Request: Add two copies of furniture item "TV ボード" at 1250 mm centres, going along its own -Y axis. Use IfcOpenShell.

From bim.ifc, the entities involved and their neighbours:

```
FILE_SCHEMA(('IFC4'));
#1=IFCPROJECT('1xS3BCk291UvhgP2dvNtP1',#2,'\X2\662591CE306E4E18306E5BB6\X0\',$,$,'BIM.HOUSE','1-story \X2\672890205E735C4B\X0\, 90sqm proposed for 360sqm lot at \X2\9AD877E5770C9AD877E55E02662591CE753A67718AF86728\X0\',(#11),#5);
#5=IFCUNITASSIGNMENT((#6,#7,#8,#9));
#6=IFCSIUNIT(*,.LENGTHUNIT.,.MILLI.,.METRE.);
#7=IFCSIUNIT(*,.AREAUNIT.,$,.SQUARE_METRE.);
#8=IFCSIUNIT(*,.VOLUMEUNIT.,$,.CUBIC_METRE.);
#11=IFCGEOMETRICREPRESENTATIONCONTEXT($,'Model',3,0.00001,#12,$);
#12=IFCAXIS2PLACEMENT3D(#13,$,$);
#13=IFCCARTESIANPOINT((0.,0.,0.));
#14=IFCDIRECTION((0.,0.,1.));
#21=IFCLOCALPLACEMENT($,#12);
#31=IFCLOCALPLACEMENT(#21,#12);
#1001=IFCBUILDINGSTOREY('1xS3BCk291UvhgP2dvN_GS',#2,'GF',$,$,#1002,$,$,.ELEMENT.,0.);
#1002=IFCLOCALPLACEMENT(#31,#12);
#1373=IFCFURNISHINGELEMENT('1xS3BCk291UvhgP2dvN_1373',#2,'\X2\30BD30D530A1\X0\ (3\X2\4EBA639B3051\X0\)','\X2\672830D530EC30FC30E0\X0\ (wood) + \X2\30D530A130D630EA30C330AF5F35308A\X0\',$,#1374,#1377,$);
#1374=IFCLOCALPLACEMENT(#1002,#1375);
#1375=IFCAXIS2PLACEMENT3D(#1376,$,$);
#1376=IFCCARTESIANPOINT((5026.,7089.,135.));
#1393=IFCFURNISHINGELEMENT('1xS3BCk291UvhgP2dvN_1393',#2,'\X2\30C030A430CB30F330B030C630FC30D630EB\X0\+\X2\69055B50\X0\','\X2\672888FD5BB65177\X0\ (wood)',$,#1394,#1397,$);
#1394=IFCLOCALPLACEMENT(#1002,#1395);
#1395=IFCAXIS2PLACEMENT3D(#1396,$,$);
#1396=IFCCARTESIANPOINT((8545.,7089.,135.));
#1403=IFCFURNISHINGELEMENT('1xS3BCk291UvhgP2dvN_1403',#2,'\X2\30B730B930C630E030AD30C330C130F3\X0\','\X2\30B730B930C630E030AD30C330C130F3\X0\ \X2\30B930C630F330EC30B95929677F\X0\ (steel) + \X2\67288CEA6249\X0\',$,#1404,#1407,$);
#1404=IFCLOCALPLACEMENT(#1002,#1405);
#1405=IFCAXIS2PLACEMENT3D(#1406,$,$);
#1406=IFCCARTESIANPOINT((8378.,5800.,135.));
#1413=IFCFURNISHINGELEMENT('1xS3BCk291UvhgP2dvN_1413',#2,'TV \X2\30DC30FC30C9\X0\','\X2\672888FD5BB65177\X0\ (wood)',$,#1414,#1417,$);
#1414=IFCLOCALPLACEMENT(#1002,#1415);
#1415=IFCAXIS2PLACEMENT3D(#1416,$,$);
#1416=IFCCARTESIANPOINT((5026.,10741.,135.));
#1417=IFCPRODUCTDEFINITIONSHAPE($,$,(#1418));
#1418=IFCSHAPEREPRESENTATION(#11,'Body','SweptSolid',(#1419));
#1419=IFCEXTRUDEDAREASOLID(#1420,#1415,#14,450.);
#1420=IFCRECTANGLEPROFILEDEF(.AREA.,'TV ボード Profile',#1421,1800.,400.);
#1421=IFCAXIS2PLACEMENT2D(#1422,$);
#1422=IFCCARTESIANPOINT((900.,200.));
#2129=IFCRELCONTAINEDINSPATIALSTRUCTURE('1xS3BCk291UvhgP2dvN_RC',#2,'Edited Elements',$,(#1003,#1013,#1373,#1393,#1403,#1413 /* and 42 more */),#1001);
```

```python
import ifcopenshell
import ifcopenshell.api.geometry
import ifcopenshell.api.root
import ifcopenshell.util.element
import ifcopenshell.util.placement
import ifcopenshell.util.unit

model = ifcopenshell.open("bim.ifc")
unit_scale = ifcopenshell.util.unit.calculate_unit_scale(model)


def reuse_history(source, copy):
    """copy_class also copies each property set's owner history, people and application; keep the originals."""
    for rel in copy.IsDefinedBy:
        if rel.is_a("IfcRelDefinesByProperties") and (history := rel.RelatingPropertyDefinition.OwnerHistory):
            rel.RelatingPropertyDefinition.OwnerHistory = source.OwnerHistory
            ifcopenshell.util.element.remove_deep2(model, history)


source = model.by_guid("1xS3BCk291UvhgP2dvN_1413")
base = ifcopenshell.util.placement.get_local_placement(source.ObjectPlacement)
step = -base[:3, 1] * 1.25 / unit_scale

for i in range(1, 3):
    copy = ifcopenshell.api.root.copy_class(model, product=source)
    copy.Representation = ifcopenshell.util.element.copy_deep(
        model, source.Representation, exclude=["IfcGeometricRepresentationContext", "IfcRepresentationMap"]
    )
    reuse_history(source, copy)
    matrix = base.copy()
    matrix[:3, 3] += i * step
    print("added at", matrix[:3, 3].round(3) + 0.0)
    ifcopenshell.api.geometry.edit_object_placement(model, product=copy, matrix=matrix, is_si=False)

model.write("bim_rev.ifc")
```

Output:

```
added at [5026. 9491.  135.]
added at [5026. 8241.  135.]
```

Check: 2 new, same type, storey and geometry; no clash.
